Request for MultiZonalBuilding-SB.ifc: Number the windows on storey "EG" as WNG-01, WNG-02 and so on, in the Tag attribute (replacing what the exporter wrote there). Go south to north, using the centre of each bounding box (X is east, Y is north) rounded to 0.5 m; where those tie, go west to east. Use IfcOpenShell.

First a look at what the model holds.

```python
import ifcopenshell
import ifcopenshell.util.element
import ifcopenshell.util.placement

model = ifcopenshell.open("MultiZonalBuilding-SB.ifc")
print(model.schema)
storey = next(s for s in model.by_type("IfcBuildingStorey") if s.Name == "EG")
windows = [e for e in ifcopenshell.util.element.get_decomposition(storey) if e.is_a("IfcWindow")]
for e in sorted(windows, key=lambda e: e.id()):
    origin = ifcopenshell.util.placement.get_local_placement(e.ObjectPlacement)[:3, 3]
    print(e.id(), e.Tag, e.Name, origin.round(2) + 0.0, sep=" | ")
```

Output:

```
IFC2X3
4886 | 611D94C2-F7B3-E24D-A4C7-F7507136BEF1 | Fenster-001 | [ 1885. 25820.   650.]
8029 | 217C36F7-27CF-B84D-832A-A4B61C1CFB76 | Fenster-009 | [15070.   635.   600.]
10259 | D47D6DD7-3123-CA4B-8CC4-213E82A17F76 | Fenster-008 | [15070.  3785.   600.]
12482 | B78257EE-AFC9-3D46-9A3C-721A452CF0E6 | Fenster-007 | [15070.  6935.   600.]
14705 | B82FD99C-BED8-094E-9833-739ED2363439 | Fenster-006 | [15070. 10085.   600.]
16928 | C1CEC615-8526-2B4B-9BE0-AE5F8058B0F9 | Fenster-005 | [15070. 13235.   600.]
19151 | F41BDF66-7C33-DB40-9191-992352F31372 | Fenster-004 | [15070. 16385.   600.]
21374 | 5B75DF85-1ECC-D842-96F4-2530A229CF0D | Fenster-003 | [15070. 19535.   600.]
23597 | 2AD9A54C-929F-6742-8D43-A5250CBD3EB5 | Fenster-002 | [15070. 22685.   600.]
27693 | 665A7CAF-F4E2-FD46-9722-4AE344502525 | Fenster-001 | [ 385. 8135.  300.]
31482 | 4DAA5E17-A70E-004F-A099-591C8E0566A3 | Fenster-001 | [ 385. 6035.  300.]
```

```python
import ifcopenshell
import ifcopenshell.geom
import ifcopenshell.util.element
import ifcopenshell.util.shape

model = ifcopenshell.open("MultiZonalBuilding-SB.ifc")
settings = ifcopenshell.geom.settings()
settings.set("use-world-coords", True)


def centre(element):
    shape = ifcopenshell.geom.create_shape(settings, element)
    return ifcopenshell.util.shape.get_bbox_centroid(shape.geometry)


storey = next(s for s in model.by_type("IfcBuildingStorey") if s.Name == "EG")
windows = [e for e in ifcopenshell.util.element.get_decomposition(storey) if e.is_a("IfcWindow")]

# Insertion points can sit at a corner or the storey origin, so sort by the geometry (in metres).
centres = {e: centre(e) for e in windows}
windows.sort(key=lambda e: (round(centres[e][1] / 0.5), centres[e][0]))

for i, e in enumerate(windows, start=1):
    number = f"WNG-{i:02d}"
    e.Tag = number
    print(e.id(), number)

model.write("MultiZonalBuilding-SB_v2.ifc")
```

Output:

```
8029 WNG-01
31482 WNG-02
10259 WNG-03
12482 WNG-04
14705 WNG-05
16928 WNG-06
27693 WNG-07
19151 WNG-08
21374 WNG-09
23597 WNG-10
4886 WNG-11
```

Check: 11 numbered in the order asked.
